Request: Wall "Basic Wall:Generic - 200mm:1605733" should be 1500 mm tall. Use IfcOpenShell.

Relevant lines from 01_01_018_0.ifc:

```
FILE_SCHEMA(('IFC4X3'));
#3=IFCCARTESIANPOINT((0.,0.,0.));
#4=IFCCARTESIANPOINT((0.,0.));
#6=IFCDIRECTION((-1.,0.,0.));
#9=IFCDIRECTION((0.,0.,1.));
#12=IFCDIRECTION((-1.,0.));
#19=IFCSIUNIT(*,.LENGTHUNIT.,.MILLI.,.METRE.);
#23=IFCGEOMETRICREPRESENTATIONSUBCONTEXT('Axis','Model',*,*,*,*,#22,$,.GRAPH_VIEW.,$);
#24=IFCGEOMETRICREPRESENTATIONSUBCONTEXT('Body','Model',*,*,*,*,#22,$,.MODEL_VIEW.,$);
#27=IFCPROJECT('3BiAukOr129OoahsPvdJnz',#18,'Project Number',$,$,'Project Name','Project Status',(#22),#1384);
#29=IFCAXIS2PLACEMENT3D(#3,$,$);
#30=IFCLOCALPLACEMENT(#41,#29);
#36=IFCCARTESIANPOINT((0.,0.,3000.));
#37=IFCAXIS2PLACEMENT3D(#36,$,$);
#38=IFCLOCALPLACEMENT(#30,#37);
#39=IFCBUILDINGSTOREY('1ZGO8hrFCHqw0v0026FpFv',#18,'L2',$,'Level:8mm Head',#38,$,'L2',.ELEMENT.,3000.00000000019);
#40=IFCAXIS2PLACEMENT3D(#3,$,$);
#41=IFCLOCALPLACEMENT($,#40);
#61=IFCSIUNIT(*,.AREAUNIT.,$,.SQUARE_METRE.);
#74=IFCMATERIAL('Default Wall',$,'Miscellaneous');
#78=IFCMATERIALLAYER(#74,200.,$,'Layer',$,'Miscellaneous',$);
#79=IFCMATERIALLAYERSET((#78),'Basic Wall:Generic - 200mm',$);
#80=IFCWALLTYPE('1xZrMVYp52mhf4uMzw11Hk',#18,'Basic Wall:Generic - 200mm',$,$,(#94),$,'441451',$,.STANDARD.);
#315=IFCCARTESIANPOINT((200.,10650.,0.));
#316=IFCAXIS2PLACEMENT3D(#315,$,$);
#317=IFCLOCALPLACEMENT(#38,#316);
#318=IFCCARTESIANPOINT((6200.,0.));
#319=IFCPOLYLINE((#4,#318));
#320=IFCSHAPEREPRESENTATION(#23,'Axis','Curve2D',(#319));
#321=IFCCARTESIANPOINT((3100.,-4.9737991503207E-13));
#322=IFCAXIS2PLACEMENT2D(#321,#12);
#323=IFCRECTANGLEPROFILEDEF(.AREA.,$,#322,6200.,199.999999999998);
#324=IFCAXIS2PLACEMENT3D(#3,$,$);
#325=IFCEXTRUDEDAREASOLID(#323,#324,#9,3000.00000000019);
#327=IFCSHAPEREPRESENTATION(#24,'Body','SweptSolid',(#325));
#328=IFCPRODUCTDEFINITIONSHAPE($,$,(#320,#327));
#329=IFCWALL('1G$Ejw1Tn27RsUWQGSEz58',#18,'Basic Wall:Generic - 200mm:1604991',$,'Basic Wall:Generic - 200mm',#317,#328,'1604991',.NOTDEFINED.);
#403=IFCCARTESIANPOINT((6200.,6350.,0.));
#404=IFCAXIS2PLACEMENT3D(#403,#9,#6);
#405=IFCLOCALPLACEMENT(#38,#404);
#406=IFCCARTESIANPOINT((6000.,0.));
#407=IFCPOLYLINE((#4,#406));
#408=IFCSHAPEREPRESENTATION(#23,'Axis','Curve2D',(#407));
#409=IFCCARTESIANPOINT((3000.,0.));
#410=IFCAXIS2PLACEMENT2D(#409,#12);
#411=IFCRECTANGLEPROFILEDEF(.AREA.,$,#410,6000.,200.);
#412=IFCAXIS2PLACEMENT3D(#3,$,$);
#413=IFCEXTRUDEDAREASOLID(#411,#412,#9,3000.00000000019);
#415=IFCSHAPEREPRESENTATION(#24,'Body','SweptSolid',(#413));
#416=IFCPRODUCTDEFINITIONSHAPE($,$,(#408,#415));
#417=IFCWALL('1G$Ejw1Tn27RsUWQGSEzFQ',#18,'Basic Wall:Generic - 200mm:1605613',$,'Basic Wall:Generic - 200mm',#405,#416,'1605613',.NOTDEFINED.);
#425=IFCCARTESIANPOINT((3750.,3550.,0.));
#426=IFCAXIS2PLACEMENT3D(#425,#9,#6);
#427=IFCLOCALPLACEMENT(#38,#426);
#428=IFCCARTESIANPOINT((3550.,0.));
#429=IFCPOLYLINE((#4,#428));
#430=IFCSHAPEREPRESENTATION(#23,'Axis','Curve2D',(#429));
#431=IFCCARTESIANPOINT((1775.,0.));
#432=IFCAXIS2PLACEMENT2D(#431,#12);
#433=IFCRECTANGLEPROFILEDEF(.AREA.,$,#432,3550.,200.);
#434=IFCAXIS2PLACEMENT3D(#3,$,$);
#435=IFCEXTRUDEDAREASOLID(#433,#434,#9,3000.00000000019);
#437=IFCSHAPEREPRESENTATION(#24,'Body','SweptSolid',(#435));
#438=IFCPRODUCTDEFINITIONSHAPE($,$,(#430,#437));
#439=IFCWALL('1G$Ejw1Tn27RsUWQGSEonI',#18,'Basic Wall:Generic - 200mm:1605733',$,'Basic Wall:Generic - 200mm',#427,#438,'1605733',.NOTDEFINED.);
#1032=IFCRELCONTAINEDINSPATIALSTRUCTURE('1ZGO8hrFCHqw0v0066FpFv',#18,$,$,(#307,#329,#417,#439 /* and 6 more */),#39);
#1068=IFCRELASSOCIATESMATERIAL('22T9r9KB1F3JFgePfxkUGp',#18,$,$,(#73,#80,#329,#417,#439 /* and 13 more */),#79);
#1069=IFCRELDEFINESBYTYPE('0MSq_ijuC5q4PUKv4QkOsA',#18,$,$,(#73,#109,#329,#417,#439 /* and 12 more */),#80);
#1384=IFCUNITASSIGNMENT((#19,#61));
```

```python
import ifcopenshell
import ifcopenshell.geom
import ifcopenshell.util.representation
import ifcopenshell.util.shape
import ifcopenshell.util.unit

model = ifcopenshell.open("01_01_018_0.ifc")
unit_scale = ifcopenshell.util.unit.calculate_unit_scale(model)
settings = ifcopenshell.geom.settings()


def volume(element):
    """Net volume in cubic metres, openings subtracted."""
    shape = ifcopenshell.geom.create_shape(settings, element)
    return ifcopenshell.util.shape.get_volume(shape.geometry)


wall = model.by_guid("1G$Ejw1Tn27RsUWQGSEonI")
before = volume(wall)

body = ifcopenshell.util.representation.get_representation(wall, "Model", "Body")
solid = body.Items[0]
old_height = solid.Depth
solid.Depth = 1.5 / unit_scale
after = volume(wall)

print(f"height {old_height:g} -> {solid.Depth:g}, volume {before:.3f} -> {after:.3f} m3")

model.write("01_01_018_0_edited.ifc")
```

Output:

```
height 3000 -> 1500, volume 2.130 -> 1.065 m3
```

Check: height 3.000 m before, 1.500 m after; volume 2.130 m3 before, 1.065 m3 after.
